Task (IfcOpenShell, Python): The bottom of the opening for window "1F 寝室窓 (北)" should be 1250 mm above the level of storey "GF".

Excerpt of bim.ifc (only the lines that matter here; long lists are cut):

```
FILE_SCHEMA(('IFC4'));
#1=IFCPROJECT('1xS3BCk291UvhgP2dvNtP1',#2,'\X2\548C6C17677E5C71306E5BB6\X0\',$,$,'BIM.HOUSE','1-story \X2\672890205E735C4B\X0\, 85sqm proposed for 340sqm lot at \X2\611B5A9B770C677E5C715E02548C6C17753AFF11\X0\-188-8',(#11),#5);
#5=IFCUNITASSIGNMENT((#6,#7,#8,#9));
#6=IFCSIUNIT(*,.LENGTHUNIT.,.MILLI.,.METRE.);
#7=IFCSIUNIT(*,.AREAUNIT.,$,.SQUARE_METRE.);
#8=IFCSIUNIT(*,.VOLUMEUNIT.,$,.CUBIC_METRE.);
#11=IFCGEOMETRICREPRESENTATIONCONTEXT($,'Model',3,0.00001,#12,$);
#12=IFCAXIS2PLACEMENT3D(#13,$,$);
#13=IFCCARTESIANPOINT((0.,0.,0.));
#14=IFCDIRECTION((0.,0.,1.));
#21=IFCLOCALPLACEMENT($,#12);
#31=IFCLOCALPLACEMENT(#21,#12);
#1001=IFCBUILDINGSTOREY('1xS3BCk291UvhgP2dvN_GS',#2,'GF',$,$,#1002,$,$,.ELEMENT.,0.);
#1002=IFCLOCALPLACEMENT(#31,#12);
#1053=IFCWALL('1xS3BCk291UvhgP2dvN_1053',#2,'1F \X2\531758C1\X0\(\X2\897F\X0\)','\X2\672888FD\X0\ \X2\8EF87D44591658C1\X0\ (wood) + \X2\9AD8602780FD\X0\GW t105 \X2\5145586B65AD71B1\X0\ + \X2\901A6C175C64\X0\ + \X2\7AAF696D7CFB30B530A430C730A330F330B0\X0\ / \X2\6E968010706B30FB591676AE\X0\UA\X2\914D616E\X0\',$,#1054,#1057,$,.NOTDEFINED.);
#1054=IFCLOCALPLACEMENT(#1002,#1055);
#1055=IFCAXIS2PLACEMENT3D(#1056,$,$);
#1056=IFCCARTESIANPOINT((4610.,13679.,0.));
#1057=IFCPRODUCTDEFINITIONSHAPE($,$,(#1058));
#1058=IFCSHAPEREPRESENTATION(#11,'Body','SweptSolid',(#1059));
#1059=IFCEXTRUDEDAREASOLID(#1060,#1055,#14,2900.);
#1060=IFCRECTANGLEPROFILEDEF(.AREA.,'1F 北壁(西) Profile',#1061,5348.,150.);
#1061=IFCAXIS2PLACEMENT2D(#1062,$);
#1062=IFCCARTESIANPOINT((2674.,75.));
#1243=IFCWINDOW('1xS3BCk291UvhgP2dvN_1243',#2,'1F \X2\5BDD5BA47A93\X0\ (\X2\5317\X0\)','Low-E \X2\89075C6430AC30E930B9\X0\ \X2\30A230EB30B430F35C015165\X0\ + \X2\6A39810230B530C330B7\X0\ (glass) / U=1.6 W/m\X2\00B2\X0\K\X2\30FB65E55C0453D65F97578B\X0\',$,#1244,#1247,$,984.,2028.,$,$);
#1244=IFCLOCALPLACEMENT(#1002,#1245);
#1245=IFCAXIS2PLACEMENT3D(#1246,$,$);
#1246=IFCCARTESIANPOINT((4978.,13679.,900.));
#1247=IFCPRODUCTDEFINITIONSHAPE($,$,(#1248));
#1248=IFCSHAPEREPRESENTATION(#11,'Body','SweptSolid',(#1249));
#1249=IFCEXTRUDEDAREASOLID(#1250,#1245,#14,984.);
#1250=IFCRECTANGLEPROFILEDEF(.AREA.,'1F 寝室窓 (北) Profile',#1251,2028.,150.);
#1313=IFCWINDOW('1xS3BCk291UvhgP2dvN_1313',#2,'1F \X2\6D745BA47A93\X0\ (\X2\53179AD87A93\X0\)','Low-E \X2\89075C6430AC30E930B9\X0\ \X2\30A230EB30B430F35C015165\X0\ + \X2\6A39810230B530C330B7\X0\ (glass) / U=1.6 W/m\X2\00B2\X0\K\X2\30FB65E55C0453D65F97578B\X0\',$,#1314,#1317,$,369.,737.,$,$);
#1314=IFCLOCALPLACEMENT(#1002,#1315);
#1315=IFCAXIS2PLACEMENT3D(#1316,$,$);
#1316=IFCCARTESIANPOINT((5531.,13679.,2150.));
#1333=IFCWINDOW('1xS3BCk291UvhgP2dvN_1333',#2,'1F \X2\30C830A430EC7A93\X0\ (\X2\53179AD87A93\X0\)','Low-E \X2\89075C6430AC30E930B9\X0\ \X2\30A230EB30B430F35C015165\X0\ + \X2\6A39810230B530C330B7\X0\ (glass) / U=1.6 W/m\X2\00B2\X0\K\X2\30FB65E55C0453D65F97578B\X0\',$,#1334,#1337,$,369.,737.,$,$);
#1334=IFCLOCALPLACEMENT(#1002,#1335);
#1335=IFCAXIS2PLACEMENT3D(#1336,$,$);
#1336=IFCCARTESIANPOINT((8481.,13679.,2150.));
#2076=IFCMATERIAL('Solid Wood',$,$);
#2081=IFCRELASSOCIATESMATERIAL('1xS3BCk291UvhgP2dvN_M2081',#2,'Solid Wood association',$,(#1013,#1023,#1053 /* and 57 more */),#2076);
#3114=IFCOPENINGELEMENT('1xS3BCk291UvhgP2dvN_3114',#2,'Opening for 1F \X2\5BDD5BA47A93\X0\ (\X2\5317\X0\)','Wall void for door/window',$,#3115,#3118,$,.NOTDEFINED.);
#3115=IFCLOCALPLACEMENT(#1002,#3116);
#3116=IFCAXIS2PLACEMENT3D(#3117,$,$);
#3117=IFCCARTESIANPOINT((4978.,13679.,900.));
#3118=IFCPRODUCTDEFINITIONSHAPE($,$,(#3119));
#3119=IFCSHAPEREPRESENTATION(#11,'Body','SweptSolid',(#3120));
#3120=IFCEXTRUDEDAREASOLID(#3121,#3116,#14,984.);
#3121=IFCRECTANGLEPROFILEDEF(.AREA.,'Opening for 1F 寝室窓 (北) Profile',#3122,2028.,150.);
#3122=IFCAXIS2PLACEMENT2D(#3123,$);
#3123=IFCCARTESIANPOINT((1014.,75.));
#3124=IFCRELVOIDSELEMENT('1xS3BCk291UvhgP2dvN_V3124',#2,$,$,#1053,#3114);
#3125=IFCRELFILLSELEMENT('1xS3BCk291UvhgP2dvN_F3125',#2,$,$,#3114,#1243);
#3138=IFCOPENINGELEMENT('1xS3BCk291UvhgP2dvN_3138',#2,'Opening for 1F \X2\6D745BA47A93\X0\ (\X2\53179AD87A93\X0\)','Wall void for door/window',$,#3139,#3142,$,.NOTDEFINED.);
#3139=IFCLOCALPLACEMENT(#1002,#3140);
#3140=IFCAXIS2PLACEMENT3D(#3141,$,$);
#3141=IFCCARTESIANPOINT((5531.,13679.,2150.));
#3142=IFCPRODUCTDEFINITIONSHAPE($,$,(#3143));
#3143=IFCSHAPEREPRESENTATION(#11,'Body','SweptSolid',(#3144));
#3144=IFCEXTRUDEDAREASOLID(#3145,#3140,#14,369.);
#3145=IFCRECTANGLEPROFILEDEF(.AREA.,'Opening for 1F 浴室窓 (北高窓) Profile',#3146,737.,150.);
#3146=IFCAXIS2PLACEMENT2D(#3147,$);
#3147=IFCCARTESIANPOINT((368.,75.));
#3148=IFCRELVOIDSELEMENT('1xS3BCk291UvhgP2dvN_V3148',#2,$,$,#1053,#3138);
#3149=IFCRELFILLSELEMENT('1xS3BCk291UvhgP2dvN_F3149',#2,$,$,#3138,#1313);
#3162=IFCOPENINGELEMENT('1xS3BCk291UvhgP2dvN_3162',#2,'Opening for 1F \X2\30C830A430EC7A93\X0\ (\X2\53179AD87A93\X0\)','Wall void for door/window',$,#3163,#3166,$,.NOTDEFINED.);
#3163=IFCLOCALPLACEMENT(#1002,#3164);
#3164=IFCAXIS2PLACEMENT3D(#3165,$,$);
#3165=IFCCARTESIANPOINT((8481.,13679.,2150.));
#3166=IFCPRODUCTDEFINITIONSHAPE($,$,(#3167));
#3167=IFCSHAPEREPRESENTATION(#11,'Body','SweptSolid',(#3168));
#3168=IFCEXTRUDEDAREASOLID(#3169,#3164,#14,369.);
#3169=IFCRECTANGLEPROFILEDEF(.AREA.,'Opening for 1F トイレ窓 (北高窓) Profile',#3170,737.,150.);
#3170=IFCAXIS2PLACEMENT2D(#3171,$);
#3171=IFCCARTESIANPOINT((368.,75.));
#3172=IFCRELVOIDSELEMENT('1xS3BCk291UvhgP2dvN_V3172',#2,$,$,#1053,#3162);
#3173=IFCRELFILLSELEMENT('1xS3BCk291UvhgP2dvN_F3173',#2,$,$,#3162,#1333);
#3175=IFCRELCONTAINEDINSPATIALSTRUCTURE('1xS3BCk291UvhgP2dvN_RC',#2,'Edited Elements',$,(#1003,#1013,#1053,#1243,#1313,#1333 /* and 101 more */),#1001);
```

```python
import numpy as np
import ifcopenshell
import ifcopenshell.api.geometry
import ifcopenshell.geom
import ifcopenshell.util.element
import ifcopenshell.util.placement
import ifcopenshell.util.shape
import ifcopenshell.util.unit

model = ifcopenshell.open("bim.ifc")
unit_scale = ifcopenshell.util.unit.calculate_unit_scale(model)

window = model.by_guid("1xS3BCk291UvhgP2dvN_1243")
opening = window.FillsVoids[0].RelatingOpeningElement
storey = ifcopenshell.util.element.get_container(window, ifc_class="IfcBuildingStorey")
level = ifcopenshell.util.placement.get_local_placement(storey.ObjectPlacement)[2, 3]

# The opening's origin need not be at the sill, so measure its lowest point.
shape = ifcopenshell.geom.create_shape(ifcopenshell.geom.settings(), opening)
bottom = ifcopenshell.util.shape.get_shape_bottom_elevation(shape, shape.geometry) / unit_scale
dz = level + 1.25 / unit_scale - bottom

shift = np.array([0.0, 0.0, dz])
# The window is not placed relative to its opening, so move both.
for product in (opening, window):
    matrix = ifcopenshell.util.placement.get_local_placement(product.ObjectPlacement)
    matrix[:3, 3] += shift
    ifcopenshell.api.geometry.edit_object_placement(model, product=product, matrix=matrix, is_si=False)

print(f"moved by {dz * unit_scale:+.3f} m")

model.write("bim_rev.ifc")
```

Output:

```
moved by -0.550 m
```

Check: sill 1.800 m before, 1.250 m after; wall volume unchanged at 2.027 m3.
